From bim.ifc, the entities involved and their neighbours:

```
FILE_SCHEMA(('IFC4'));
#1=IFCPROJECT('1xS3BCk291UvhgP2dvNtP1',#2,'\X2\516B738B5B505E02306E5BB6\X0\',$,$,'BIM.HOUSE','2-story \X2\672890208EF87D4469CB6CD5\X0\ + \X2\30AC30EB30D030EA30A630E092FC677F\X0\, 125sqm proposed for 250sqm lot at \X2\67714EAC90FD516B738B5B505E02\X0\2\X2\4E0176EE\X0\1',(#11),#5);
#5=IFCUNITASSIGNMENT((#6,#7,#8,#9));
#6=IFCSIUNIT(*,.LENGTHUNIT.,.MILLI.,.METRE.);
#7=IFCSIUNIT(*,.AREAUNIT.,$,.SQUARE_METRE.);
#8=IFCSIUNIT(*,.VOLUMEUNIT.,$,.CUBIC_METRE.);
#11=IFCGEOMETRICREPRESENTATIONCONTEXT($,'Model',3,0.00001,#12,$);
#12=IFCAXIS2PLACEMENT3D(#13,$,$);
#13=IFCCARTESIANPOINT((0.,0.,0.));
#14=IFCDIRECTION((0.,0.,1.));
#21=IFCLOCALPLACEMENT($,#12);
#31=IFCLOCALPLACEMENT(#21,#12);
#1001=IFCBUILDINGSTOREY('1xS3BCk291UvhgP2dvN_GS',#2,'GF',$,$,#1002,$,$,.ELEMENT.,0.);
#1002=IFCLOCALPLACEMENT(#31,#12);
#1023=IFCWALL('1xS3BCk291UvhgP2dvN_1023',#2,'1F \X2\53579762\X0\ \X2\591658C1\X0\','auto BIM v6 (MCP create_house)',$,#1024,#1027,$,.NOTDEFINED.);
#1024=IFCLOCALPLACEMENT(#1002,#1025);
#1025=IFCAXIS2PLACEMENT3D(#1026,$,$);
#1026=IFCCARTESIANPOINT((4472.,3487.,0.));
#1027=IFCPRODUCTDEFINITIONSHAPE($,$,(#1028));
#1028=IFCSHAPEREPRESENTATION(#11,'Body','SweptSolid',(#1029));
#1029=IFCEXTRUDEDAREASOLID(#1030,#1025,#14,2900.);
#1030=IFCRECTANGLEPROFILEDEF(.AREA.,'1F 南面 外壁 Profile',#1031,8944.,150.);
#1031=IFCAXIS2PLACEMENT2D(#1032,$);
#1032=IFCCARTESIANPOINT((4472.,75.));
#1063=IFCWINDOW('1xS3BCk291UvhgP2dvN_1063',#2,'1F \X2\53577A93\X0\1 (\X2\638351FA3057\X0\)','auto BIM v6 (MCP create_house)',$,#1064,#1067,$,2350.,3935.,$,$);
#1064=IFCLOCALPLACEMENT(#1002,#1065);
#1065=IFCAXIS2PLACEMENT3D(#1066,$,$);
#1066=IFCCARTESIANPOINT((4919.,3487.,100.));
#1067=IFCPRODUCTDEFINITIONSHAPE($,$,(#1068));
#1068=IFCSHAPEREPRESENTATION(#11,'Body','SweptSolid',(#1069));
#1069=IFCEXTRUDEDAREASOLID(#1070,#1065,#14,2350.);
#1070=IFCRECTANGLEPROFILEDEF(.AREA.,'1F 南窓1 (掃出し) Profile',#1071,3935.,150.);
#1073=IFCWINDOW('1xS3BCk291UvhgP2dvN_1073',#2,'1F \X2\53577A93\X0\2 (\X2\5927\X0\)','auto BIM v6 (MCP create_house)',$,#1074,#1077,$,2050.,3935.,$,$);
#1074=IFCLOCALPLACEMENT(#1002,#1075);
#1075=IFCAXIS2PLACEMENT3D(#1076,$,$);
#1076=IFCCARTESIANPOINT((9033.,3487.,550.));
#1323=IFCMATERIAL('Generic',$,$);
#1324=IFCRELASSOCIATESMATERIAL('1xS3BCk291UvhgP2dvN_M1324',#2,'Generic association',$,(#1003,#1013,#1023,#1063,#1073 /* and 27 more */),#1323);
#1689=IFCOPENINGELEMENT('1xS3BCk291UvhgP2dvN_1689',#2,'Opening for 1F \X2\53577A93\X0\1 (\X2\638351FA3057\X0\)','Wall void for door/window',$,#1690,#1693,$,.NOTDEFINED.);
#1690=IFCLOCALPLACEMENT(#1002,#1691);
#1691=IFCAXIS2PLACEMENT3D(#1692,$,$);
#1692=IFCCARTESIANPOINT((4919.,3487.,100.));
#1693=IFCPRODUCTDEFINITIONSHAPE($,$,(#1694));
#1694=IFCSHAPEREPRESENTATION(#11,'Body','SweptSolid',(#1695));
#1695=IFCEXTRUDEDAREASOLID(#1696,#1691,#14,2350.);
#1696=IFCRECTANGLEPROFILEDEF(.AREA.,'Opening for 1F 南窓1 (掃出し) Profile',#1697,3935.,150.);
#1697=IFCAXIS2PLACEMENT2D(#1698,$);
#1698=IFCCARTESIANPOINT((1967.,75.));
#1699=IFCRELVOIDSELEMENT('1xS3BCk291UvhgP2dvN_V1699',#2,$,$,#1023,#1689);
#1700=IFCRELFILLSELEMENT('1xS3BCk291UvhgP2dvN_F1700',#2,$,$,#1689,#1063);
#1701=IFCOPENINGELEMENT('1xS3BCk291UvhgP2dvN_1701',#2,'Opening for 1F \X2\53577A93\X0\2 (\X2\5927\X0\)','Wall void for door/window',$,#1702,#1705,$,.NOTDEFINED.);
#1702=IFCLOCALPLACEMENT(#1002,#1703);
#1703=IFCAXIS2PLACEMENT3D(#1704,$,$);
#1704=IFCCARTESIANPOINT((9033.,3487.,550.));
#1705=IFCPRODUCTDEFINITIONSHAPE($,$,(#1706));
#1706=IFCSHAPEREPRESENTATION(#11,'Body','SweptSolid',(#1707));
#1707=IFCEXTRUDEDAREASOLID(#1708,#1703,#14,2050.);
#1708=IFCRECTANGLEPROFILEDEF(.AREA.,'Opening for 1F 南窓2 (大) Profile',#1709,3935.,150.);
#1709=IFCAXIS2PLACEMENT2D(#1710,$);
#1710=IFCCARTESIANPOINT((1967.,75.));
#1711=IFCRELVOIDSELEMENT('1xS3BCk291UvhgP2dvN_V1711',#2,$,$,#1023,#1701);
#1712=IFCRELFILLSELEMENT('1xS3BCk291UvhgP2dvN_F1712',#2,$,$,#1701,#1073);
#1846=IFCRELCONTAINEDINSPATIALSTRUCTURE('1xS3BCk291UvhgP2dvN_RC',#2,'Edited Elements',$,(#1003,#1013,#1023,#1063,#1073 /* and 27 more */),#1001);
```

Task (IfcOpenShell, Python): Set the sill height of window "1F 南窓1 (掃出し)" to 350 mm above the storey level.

```python
import numpy as np
import ifcopenshell
import ifcopenshell.api.geometry
import ifcopenshell.geom
import ifcopenshell.util.element
import ifcopenshell.util.placement
import ifcopenshell.util.shape
import ifcopenshell.util.unit

model = ifcopenshell.open("bim.ifc")
unit_scale = ifcopenshell.util.unit.calculate_unit_scale(model)

window = model.by_guid("1xS3BCk291UvhgP2dvN_1063")
opening = window.FillsVoids[0].RelatingOpeningElement
storey = ifcopenshell.util.element.get_container(window, ifc_class="IfcBuildingStorey")
level = ifcopenshell.util.placement.get_local_placement(storey.ObjectPlacement)[2, 3]

# The opening's origin need not be at the sill, so measure its lowest point.
shape = ifcopenshell.geom.create_shape(ifcopenshell.geom.settings(), opening)
bottom = ifcopenshell.util.shape.get_shape_bottom_elevation(shape, shape.geometry) / unit_scale
dz = level + 0.35 / unit_scale - bottom

shift = np.array([0.0, 0.0, dz])
# The window is not placed relative to its opening, so move both.
for product in (opening, window):
    matrix = ifcopenshell.util.placement.get_local_placement(product.ObjectPlacement)
    matrix[:3, 3] += shift
    ifcopenshell.api.geometry.edit_object_placement(model, product=product, matrix=matrix, is_si=False)

print(f"moved by {dz * unit_scale:+.3f} m")

model.write("bim_updated.ifc")
```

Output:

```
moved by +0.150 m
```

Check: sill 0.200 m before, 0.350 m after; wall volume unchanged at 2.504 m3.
